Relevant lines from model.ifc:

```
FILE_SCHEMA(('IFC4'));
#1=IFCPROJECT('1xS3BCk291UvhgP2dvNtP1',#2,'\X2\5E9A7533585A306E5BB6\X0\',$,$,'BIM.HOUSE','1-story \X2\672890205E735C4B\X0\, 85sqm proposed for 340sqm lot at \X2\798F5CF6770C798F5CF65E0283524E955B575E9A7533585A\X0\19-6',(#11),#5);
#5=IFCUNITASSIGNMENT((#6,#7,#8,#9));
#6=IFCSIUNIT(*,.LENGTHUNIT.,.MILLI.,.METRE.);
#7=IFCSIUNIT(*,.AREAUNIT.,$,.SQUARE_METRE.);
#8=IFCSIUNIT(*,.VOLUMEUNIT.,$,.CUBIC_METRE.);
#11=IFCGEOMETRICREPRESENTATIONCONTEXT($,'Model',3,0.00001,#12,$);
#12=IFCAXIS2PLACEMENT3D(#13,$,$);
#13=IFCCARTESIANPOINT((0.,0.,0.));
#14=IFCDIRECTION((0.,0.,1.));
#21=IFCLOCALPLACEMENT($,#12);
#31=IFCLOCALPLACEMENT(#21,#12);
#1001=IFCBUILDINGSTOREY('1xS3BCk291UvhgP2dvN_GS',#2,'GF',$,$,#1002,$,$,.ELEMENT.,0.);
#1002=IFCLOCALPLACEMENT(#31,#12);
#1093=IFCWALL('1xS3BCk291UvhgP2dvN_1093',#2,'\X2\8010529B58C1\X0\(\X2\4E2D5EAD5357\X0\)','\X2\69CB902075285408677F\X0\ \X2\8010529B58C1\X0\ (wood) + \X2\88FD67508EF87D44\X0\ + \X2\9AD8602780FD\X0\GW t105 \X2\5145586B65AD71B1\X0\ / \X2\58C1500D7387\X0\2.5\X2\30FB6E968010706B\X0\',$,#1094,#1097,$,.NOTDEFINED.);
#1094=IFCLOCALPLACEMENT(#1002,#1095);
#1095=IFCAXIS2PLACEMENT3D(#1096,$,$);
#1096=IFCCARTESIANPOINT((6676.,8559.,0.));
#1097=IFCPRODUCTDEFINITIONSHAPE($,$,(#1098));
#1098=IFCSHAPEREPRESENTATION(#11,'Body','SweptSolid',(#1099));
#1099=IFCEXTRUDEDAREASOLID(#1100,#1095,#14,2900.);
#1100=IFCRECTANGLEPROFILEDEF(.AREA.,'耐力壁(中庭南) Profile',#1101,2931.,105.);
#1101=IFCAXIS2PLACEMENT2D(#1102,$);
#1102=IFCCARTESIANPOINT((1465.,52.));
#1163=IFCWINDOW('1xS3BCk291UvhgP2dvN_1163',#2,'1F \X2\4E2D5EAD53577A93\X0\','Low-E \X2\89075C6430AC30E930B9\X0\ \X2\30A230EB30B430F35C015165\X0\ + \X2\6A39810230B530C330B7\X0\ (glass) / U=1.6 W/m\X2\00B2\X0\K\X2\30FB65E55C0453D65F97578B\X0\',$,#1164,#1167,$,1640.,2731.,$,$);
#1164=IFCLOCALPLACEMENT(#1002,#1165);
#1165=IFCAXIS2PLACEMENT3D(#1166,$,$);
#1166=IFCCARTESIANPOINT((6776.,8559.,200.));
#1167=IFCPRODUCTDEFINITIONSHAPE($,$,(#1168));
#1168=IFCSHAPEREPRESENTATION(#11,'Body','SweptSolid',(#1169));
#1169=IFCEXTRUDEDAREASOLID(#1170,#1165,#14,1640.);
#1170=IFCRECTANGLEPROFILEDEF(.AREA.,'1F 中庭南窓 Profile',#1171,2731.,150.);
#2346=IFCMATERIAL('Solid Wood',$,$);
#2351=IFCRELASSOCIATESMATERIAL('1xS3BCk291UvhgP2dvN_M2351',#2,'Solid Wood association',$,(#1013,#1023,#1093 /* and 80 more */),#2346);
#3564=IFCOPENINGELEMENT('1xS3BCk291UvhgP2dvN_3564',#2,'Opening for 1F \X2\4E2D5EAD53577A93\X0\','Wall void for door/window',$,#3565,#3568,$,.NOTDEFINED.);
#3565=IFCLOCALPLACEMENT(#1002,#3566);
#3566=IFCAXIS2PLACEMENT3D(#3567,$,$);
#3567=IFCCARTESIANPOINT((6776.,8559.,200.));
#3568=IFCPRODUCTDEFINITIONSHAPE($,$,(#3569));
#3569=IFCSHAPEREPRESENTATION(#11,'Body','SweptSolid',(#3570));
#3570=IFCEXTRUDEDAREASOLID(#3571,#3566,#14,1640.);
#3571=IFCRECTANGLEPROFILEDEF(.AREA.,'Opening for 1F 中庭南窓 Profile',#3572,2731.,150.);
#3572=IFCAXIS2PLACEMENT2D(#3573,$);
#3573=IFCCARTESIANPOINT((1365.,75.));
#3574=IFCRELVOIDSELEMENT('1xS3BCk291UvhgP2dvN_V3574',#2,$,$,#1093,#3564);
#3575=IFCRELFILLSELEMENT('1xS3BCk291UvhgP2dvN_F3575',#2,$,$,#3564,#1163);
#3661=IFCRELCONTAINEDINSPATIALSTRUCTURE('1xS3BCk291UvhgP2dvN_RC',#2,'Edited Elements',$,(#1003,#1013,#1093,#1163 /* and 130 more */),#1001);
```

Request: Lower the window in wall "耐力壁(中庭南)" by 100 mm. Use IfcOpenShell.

```python
import numpy as np
import ifcopenshell
import ifcopenshell.api.geometry
import ifcopenshell.util.placement
import ifcopenshell.util.unit

model = ifcopenshell.open("model.ifc")
unit_scale = ifcopenshell.util.unit.calculate_unit_scale(model)

window = model.by_guid("1xS3BCk291UvhgP2dvN_1163")
opening = window.FillsVoids[0].RelatingOpeningElement
dz = -0.1 / unit_scale

shift = np.array([0.0, 0.0, dz])
# The window is not placed relative to its opening, so move both.
for product in (opening, window):
    matrix = ifcopenshell.util.placement.get_local_placement(product.ObjectPlacement)
    matrix[:3, 3] += shift
    ifcopenshell.api.geometry.edit_object_placement(model, product=product, matrix=matrix, is_si=False)

print(f"moved by {dz * unit_scale:+.3f} m")

model.write("model_v2.ifc")
```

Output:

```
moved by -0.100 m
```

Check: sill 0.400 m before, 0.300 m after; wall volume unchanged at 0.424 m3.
